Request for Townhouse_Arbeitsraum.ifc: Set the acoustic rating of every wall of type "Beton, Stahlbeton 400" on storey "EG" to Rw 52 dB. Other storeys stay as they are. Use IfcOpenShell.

First a look at what the model holds.

```python
import ifcopenshell
import ifcopenshell.util.element

model = ifcopenshell.open("Townhouse_Arbeitsraum.ifc")
print(model.schema)
storey = next(s for s in model.by_type("IfcBuildingStorey") if s.Name == "EG")
walls = [e for e in ifcopenshell.util.element.get_decomposition(storey) if e.is_a("IfcWall")]
seen = {}
for e in walls:
    element_type = ifcopenshell.util.element.get_type(e)
    key = (element_type.Name if element_type != e and element_type else None, ifcopenshell.util.element.get_pset(e, "Pset_WallCommon", "AcousticRating"))
    seen[key] = seen.get(key, 0) + 1
for (name, value), count in sorted(seen.items(), key=str):
    print(count, "x", name, "|", value)
```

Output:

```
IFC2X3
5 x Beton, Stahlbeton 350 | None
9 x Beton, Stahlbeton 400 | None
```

```python
import ifcopenshell
import ifcopenshell.api.pset
import ifcopenshell.util.element

model = ifcopenshell.open("Townhouse_Arbeitsraum.ifc")

storey = next(s for s in model.by_type("IfcBuildingStorey") if s.Name == "EG")
walls = [e for e in ifcopenshell.util.element.get_decomposition(storey) if e.is_a("IfcWall")]

count = 0
for e in walls:
    element_type = ifcopenshell.util.element.get_type(e)
    if element_type in (None, e) or element_type.Name != "Beton, Stahlbeton 400":
        continue
    # add_pset returns the element's existing set when there is one.
    pset = ifcopenshell.api.pset.add_pset(model, product=e, name="Pset_WallCommon")
    ifcopenshell.api.pset.edit_pset(model, pset=pset, properties={"AcousticRating": "Rw 52 dB"})
    count += 1

print(count, "walls updated")

model.write("Townhouse_Arbeitsraum_edited.ifc")
```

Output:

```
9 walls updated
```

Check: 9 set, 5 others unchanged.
